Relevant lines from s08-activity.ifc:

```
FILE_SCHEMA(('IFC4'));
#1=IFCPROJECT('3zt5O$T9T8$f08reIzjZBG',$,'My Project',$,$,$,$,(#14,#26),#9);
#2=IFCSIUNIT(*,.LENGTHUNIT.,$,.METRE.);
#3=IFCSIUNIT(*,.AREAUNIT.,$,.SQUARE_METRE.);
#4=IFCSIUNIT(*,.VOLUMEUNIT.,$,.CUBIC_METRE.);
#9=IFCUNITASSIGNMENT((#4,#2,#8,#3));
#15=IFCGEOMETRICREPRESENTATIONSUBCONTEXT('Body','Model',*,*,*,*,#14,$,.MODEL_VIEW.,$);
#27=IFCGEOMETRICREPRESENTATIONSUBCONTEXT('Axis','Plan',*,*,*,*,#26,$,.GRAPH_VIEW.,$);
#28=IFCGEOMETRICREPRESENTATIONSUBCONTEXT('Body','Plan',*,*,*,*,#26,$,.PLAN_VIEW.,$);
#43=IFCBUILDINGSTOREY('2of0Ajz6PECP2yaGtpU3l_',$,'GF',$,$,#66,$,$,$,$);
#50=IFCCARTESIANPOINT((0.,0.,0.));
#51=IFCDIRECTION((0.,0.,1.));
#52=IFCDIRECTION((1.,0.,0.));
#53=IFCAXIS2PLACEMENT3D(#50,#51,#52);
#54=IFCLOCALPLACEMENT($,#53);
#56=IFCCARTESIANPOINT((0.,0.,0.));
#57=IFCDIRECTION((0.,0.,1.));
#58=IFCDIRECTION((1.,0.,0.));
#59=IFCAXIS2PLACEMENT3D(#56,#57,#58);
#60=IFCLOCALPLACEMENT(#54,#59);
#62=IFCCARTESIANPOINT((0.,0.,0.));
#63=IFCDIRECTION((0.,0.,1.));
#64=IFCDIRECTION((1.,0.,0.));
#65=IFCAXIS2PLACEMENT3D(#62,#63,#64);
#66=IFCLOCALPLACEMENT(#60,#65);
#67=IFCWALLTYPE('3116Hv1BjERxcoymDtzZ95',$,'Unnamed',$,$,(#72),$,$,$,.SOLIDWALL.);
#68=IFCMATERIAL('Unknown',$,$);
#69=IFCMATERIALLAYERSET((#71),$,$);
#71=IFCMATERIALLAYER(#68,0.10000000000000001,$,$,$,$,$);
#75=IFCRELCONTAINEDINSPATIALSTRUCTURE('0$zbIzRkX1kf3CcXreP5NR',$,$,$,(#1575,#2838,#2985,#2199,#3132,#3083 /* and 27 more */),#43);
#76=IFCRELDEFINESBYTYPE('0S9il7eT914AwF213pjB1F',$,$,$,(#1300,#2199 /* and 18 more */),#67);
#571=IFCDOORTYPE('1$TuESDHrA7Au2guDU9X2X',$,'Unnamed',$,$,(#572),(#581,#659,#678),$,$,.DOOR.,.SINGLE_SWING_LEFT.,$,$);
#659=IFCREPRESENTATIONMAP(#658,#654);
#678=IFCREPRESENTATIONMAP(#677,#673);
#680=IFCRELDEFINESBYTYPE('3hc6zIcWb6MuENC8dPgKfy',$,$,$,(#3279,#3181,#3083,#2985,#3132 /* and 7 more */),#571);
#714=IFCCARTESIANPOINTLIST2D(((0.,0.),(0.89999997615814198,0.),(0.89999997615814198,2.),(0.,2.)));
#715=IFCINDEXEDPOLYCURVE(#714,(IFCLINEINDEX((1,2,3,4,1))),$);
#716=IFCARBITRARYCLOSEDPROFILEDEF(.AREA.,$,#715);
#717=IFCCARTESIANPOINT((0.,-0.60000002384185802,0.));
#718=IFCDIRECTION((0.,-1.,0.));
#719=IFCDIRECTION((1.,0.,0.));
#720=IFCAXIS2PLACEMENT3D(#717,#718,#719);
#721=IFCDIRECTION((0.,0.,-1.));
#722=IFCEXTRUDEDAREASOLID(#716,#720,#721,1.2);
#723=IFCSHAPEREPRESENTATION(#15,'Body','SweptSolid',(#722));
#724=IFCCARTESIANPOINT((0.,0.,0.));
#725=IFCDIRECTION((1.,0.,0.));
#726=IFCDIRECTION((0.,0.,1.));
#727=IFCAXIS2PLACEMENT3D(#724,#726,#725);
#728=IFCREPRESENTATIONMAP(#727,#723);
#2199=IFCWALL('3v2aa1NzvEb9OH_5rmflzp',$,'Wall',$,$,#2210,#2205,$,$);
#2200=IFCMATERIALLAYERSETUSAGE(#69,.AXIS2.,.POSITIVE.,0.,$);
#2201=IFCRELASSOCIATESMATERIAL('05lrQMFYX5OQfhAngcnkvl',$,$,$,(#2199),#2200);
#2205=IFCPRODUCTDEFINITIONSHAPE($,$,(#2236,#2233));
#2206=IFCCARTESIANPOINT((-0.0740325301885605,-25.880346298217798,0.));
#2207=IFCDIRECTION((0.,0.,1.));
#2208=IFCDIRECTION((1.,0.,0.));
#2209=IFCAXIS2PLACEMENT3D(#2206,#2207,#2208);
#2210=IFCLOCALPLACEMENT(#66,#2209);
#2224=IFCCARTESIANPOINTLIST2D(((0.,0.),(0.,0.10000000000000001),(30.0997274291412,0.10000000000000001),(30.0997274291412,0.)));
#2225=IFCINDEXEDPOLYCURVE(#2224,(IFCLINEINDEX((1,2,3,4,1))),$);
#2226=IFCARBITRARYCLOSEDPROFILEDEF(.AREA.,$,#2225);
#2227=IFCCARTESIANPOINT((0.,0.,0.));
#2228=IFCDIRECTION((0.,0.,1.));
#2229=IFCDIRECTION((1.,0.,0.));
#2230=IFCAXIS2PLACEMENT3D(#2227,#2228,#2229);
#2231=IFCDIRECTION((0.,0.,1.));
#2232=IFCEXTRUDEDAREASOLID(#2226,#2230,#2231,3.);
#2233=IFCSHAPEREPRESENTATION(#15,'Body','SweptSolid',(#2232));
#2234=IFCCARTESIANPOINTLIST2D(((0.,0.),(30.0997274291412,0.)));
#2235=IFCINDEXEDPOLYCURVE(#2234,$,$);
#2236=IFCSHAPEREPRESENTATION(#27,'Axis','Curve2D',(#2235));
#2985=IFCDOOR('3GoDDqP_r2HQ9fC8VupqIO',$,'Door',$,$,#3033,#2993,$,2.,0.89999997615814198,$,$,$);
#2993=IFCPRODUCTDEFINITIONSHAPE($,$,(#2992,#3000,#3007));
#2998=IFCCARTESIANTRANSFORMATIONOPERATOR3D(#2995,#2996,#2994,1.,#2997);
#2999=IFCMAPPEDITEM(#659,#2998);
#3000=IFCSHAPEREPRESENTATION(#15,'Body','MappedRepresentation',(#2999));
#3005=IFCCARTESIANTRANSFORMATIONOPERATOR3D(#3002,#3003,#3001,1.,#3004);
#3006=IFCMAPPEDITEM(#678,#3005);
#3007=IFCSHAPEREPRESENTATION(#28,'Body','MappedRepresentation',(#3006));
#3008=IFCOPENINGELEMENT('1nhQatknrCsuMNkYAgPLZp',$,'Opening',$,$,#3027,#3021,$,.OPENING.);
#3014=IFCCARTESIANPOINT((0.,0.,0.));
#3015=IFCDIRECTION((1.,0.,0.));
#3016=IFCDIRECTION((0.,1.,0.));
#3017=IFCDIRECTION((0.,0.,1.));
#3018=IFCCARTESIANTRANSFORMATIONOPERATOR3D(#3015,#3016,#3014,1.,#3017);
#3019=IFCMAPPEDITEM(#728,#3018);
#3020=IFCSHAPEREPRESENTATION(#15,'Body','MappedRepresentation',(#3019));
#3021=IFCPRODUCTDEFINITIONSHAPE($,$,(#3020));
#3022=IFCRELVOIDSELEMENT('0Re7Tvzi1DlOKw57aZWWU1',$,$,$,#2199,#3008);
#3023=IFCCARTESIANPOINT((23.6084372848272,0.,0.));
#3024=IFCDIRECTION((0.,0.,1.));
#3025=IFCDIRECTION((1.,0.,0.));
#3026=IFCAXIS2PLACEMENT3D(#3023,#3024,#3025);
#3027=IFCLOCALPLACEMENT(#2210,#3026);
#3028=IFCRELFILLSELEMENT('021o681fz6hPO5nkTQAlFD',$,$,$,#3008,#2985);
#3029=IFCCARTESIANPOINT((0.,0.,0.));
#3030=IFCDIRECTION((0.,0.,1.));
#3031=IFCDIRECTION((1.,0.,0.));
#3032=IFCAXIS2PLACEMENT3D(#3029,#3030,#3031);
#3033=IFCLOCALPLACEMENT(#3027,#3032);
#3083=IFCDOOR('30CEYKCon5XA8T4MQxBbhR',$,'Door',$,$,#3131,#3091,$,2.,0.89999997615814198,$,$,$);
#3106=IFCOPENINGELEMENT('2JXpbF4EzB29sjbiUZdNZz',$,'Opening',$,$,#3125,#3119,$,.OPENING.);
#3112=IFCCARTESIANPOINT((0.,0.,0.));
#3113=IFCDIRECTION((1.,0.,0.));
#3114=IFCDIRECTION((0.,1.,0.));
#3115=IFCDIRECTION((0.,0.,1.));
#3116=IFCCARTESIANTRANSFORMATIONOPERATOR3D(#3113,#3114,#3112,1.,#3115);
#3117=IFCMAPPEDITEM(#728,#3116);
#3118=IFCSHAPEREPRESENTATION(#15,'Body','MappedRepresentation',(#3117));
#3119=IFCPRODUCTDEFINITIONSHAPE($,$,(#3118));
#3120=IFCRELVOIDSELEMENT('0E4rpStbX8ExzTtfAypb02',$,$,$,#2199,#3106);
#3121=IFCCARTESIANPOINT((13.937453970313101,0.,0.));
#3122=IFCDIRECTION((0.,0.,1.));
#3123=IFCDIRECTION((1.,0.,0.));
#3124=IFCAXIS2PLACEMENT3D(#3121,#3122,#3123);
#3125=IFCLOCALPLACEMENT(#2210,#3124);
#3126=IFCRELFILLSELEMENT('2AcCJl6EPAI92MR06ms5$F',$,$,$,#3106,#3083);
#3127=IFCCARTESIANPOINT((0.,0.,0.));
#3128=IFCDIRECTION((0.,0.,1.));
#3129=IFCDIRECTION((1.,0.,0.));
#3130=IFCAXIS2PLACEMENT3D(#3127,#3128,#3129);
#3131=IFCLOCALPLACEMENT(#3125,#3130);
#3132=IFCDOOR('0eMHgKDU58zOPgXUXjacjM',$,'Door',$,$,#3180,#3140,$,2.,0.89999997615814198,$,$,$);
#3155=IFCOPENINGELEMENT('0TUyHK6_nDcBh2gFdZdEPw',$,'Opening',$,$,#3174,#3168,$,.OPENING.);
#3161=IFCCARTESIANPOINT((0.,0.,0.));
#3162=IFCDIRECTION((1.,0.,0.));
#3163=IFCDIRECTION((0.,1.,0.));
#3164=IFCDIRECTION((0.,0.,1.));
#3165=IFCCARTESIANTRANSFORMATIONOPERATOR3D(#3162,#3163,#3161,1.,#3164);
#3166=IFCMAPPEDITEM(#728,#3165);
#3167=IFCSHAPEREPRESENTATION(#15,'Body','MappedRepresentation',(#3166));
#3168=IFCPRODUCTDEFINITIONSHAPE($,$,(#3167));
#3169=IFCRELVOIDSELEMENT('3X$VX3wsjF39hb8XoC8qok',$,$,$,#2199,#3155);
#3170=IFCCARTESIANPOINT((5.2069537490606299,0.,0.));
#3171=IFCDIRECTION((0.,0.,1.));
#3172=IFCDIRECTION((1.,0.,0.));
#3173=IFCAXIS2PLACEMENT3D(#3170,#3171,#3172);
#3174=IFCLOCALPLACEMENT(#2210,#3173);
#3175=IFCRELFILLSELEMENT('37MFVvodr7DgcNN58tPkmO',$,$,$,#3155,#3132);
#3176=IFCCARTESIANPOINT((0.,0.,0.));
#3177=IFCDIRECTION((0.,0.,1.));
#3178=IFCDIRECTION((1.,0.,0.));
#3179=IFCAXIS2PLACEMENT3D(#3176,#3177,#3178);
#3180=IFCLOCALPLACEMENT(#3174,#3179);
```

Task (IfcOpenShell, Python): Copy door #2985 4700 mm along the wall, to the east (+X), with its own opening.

```python
import ifcopenshell
import ifcopenshell.api.feature
import ifcopenshell.api.geometry
import ifcopenshell.api.root
import ifcopenshell.geom
import ifcopenshell.util.element
import ifcopenshell.util.placement
import ifcopenshell.util.shape
import ifcopenshell.util.unit

model = ifcopenshell.open("s08-activity.ifc")
unit_scale = ifcopenshell.util.unit.calculate_unit_scale(model)
settings = ifcopenshell.geom.settings()


def volume(element):
    """Net volume in cubic metres, openings subtracted."""
    shape = ifcopenshell.geom.create_shape(settings, element)
    return ifcopenshell.util.shape.get_volume(shape.geometry)


door = model.by_id(2985)
opening = door.FillsVoids[0].RelatingOpeningElement
wall = opening.VoidsElements[0].RelatingBuildingElement
before = volume(wall)
shift = ifcopenshell.util.placement.get_local_placement(wall.ObjectPlacement)[:3, 0] * 4.7 / unit_scale

# copy_class copies the void relationship, type, container and properties, but no geometry.
new_opening = ifcopenshell.api.root.copy_class(model, product=opening)
new_opening.Representation = ifcopenshell.util.element.copy_deep(
    model, opening.Representation, exclude=["IfcGeometricRepresentationContext", "IfcRepresentationMap"]
)
new_door = ifcopenshell.api.root.copy_class(model, product=door)
new_door.Representation = ifcopenshell.util.element.copy_deep(
    model, door.Representation, exclude=["IfcGeometricRepresentationContext", "IfcRepresentationMap"]
)
ifcopenshell.api.feature.add_filling(model, opening=new_opening, element=new_door)

for old, new in ((opening, new_opening), (door, new_door)):
    matrix = ifcopenshell.util.placement.get_local_placement(old.ObjectPlacement)
    matrix[:3, 3] += shift
    ifcopenshell.api.geometry.edit_object_placement(model, product=new, matrix=matrix, is_si=False)

after = volume(wall)

print(f"wall volume {before:.3f} -> {after:.3f} m3")

model.write("s08-activity_rev.ifc")
```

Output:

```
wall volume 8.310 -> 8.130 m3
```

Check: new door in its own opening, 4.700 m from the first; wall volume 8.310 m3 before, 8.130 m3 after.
